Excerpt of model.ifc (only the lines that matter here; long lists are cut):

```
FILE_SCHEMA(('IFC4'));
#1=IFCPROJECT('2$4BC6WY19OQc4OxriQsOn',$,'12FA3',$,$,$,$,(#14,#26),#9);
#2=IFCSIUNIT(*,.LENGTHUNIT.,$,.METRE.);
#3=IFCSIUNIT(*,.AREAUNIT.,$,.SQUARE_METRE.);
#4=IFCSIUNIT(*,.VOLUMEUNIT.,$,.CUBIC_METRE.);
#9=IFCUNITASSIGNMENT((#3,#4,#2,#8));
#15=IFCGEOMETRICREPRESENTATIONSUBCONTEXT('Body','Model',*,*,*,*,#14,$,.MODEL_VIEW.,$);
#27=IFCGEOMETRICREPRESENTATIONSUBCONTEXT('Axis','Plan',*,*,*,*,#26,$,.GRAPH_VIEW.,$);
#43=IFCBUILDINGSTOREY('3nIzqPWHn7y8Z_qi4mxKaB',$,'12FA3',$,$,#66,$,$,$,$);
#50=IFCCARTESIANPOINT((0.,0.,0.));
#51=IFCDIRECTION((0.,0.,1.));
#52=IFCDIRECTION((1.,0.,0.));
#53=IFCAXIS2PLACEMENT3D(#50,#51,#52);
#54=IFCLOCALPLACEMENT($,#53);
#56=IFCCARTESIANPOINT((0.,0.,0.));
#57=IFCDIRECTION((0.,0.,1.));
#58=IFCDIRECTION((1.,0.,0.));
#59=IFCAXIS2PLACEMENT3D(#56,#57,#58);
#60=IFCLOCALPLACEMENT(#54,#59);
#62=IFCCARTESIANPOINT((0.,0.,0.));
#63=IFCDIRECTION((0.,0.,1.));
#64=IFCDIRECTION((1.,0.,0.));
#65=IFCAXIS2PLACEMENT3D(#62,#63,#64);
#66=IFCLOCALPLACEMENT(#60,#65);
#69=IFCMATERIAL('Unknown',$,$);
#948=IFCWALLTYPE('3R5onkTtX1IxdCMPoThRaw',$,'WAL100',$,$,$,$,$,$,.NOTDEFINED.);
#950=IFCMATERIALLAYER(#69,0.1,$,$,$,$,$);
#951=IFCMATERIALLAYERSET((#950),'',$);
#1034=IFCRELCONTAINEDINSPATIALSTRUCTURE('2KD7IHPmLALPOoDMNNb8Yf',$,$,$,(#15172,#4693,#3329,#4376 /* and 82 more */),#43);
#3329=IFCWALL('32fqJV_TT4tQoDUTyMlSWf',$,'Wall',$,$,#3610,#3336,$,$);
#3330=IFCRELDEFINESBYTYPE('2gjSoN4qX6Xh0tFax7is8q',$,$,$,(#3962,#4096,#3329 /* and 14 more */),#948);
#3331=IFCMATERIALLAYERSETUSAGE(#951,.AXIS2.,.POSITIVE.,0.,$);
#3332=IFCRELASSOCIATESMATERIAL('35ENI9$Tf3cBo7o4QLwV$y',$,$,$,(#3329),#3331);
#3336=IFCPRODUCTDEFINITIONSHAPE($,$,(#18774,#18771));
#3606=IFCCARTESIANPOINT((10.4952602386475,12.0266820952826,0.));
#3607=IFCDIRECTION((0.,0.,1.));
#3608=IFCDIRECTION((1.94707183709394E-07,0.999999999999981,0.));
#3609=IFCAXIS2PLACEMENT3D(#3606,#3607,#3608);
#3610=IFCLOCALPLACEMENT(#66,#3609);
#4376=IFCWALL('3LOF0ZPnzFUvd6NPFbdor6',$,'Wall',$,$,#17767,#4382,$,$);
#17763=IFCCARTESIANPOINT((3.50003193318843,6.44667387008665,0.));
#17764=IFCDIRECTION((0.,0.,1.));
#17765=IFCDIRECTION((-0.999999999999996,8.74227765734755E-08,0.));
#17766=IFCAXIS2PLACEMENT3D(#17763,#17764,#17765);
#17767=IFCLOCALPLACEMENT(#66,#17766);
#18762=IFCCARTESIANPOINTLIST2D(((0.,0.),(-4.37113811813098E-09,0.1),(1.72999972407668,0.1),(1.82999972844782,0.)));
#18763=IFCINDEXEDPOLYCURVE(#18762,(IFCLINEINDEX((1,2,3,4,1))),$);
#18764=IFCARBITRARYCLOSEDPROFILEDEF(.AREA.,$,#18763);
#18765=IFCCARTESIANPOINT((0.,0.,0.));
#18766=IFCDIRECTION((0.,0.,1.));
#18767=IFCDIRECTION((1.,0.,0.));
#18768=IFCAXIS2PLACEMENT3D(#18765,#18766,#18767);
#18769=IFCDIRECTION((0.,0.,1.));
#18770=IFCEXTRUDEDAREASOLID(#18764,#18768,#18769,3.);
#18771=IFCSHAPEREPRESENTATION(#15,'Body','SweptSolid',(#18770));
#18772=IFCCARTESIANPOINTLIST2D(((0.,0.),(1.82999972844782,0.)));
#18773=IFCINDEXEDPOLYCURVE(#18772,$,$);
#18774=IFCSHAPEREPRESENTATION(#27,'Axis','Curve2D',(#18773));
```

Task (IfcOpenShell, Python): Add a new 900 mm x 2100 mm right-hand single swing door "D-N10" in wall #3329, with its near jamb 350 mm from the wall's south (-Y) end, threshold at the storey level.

```python
import numpy as np
import ifcopenshell
import ifcopenshell.api.feature
import ifcopenshell.api.geometry
import ifcopenshell.api.root
import ifcopenshell.api.spatial
import ifcopenshell.geom
import ifcopenshell.util.element
import ifcopenshell.util.placement
import ifcopenshell.util.representation
import ifcopenshell.util.shape
import ifcopenshell.util.unit

model = ifcopenshell.open("model.ifc")
unit_scale = ifcopenshell.util.unit.calculate_unit_scale(model)
settings = ifcopenshell.geom.settings()


def volume(element):
    """Net volume in cubic metres, openings subtracted."""
    shape = ifcopenshell.geom.create_shape(settings, element)
    return ifcopenshell.util.shape.get_volume(shape.geometry)


wall = model.by_id(3329)
storey = ifcopenshell.util.element.get_container(wall, ifc_class="IfcBuildingStorey")
context = ifcopenshell.util.representation.get_context(model, "Model", "Body", "MODEL_VIEW")
before = volume(wall)

width, height, from_end, sill = 0.9, 2.1, 0.35, 0.0  # metres

# The wall runs along its own X axis, and the end named is its -X end.
wall_shape = ifcopenshell.geom.create_shape(settings, wall)
x, y, z = ifcopenshell.util.shape.get_vertices(wall_shape.geometry).T
start = x.min() + from_end
face, thickness = float(y.min()), float(y.max() - y.min())
wall_matrix = ifcopenshell.util.placement.get_local_placement(wall.ObjectPlacement)
level = ifcopenshell.util.placement.get_local_placement(storey.ObjectPlacement)[2, 3]


def in_wall(x, y):
    """Placement at x, y metres in the wall's axes, at sill height."""
    matrix = wall_matrix.copy()
    matrix[:, 3] = wall_matrix @ np.array([x / unit_scale, y / unit_scale, 0.0, 1.0])
    matrix[2, 3] = level + sill / unit_scale
    return matrix


# Opening: a box that overshoots both wall faces by 50 mm.
opening = ifcopenshell.api.root.create_entity(model, ifc_class="IfcOpeningElement", predefined_type="OPENING")
box = ifcopenshell.api.geometry.add_wall_representation(
    model, context=context, length=width, height=height, thickness=thickness + 0.1
)
ifcopenshell.api.geometry.assign_representation(model, product=opening, representation=box)
ifcopenshell.api.geometry.edit_object_placement(model, product=opening, matrix=in_wall(start, face - 0.05), is_si=False)
ifcopenshell.api.feature.add_feature(model, feature=opening, element=wall)

door = ifcopenshell.api.root.create_entity(model, ifc_class="IfcDoor", name="D-N10", predefined_type="DOOR")
door.OverallWidth, door.OverallHeight = width / unit_scale, height / unit_scale
door.OperationType = "SINGLE_SWING_RIGHT"
body = ifcopenshell.api.geometry.add_door_representation(
    model,
    context=context,
    overall_width=door.OverallWidth,
    overall_height=door.OverallHeight,
    operation_type="SINGLE_SWING_RIGHT",
    lining_properties={"LiningDepth": thickness / unit_scale, "ThresholdDepth": thickness / unit_scale},
)
ifcopenshell.api.geometry.assign_representation(model, product=door, representation=body)
ifcopenshell.api.spatial.assign_container(model, products=[door], relating_structure=storey)
ifcopenshell.api.feature.add_filling(model, opening=opening, element=door)

# The lining spans the wall, so the door starts at the wall face.
ifcopenshell.api.geometry.edit_object_placement(model, product=door, matrix=in_wall(start, face), is_si=False)

after = volume(wall)

print(f"wall volume {before:.3f} -> {after:.3f} m3")

model.write("model_edited.ifc")
```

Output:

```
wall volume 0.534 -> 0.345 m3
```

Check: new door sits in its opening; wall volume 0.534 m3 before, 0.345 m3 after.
